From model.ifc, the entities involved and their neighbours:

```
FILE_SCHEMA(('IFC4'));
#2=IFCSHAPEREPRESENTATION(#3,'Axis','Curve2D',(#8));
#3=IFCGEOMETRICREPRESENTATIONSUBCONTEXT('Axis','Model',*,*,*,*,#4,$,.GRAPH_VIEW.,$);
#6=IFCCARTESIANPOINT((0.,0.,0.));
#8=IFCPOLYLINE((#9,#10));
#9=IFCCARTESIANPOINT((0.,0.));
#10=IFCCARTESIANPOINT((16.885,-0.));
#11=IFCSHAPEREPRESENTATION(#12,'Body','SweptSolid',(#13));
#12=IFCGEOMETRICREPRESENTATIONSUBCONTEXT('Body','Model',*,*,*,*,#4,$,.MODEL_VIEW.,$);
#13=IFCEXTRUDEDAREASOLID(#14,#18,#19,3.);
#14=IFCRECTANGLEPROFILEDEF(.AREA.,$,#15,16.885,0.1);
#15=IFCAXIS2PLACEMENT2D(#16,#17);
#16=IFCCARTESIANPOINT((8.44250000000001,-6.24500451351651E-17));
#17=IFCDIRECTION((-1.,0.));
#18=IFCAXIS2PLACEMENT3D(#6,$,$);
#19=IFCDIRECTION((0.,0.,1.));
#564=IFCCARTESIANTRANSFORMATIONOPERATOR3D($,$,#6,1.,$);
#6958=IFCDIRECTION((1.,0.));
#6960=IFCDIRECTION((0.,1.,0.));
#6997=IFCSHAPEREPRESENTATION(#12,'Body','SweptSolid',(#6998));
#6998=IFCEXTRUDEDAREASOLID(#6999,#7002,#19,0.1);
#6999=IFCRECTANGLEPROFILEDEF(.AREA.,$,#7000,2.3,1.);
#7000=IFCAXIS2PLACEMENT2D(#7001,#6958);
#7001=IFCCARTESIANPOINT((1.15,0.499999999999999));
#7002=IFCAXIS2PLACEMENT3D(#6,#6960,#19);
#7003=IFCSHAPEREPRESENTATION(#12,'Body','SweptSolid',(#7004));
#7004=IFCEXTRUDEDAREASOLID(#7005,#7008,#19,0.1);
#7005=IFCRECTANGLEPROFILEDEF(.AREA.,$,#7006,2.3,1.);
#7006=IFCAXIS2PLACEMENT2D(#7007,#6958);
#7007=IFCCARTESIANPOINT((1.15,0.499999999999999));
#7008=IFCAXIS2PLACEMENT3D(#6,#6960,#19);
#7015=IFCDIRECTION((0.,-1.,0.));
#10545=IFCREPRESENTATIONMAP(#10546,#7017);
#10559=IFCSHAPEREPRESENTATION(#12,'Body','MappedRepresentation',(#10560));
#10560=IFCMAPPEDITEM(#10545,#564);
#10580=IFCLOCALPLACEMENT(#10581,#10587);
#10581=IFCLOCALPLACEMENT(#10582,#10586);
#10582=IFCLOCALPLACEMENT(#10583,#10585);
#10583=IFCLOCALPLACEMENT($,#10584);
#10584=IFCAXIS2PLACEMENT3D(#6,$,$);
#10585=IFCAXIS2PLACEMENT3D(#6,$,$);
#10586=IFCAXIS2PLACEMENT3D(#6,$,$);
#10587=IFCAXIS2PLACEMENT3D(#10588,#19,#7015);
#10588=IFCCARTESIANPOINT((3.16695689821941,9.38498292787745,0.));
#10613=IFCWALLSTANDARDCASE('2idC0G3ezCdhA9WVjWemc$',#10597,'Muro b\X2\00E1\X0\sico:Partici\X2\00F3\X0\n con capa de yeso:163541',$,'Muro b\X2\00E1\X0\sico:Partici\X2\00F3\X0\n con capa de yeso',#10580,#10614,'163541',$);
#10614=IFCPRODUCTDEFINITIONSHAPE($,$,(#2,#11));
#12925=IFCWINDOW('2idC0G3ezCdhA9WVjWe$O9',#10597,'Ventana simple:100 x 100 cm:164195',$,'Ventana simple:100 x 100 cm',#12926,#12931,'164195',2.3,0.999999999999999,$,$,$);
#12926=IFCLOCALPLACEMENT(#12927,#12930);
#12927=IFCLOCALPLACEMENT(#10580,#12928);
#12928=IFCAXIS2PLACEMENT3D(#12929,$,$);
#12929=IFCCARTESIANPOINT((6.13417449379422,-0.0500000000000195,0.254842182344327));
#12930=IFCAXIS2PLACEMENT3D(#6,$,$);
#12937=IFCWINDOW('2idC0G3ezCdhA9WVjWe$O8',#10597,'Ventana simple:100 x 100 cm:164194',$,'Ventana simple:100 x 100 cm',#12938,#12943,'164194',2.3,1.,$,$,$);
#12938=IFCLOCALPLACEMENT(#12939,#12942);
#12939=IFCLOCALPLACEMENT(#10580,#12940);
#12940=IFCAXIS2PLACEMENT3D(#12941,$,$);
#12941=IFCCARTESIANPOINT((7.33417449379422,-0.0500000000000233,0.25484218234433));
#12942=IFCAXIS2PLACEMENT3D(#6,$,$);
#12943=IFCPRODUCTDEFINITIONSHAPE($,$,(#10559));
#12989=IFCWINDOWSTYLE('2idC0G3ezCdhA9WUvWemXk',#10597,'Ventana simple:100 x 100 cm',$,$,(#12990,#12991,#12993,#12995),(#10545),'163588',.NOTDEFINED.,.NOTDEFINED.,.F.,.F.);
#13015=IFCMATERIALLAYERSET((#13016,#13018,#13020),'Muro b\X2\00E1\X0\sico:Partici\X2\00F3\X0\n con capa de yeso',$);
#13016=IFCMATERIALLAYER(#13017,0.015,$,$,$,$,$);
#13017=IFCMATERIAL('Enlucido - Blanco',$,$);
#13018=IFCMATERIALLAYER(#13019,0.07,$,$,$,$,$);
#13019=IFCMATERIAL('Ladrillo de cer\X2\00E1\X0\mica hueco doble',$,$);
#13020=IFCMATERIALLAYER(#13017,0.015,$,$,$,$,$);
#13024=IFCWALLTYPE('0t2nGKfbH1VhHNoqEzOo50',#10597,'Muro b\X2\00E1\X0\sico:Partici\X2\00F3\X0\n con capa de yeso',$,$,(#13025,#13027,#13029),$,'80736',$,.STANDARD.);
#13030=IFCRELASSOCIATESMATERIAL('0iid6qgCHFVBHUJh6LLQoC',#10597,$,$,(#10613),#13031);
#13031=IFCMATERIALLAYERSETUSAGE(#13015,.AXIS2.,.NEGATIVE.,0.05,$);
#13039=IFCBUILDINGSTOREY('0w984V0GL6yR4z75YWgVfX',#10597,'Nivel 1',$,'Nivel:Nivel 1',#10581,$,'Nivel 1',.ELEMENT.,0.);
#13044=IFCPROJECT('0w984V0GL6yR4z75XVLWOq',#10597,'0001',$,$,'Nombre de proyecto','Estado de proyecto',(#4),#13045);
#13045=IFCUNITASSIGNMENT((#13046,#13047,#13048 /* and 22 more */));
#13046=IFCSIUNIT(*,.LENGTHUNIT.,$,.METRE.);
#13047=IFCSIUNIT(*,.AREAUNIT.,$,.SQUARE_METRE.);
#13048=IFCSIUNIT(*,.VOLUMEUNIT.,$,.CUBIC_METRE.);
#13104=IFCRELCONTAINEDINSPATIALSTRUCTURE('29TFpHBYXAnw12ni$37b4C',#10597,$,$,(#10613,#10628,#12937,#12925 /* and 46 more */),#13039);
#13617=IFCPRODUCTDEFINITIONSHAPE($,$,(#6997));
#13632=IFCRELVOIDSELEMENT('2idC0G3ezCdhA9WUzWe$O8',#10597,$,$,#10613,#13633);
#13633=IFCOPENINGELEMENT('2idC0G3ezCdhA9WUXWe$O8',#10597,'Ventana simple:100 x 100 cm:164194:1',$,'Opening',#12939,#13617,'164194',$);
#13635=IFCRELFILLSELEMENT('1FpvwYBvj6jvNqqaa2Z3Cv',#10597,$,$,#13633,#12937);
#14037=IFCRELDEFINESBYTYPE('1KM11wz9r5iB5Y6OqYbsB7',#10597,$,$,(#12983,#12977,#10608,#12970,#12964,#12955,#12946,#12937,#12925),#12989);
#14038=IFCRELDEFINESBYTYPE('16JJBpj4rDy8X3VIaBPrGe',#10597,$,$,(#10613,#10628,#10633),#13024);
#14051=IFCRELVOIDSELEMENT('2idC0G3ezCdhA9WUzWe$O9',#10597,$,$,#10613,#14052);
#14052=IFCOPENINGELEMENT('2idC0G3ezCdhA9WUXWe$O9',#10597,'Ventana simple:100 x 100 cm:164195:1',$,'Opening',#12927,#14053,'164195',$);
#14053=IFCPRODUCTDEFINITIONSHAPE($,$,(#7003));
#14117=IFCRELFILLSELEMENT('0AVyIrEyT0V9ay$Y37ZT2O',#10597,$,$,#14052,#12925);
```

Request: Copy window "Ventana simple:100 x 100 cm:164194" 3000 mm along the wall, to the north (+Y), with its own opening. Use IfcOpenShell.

```python
import ifcopenshell
import ifcopenshell.api.feature
import ifcopenshell.api.geometry
import ifcopenshell.api.root
import ifcopenshell.geom
import ifcopenshell.util.element
import ifcopenshell.util.placement
import ifcopenshell.util.shape

model = ifcopenshell.open("model.ifc")
settings = ifcopenshell.geom.settings()


def volume(element):
    """Net volume in cubic metres, openings subtracted."""
    shape = ifcopenshell.geom.create_shape(settings, element)
    return ifcopenshell.util.shape.get_volume(shape.geometry)


def reuse_history(source, copy):
    """copy_class also copies each property set's owner history, people and application; keep the originals."""
    for rel in copy.IsDefinedBy:
        if rel.is_a("IfcRelDefinesByProperties") and (history := rel.RelatingPropertyDefinition.OwnerHistory):
            rel.RelatingPropertyDefinition.OwnerHistory = source.OwnerHistory
            ifcopenshell.util.element.remove_deep2(model, history)


window = model.by_guid("2idC0G3ezCdhA9WVjWe$O8")
opening = window.FillsVoids[0].RelatingOpeningElement
wall = opening.VoidsElements[0].RelatingBuildingElement
before = volume(wall)
shift = ifcopenshell.util.placement.get_local_placement(wall.ObjectPlacement)[:3, 0] * -3.0

# copy_class copies the void relationship, type, container and properties, but no geometry.
new_opening = ifcopenshell.api.root.copy_class(model, product=opening)
new_opening.Representation = ifcopenshell.util.element.copy_deep(
    model, opening.Representation, exclude=["IfcGeometricRepresentationContext", "IfcRepresentationMap"]
)
new_opening.Name = "Ventana simple:100 x 100 cm"
new_opening.Tag = None
new_window = ifcopenshell.api.root.copy_class(model, product=window)
new_window.Representation = ifcopenshell.util.element.copy_deep(
    model, window.Representation, exclude=["IfcGeometricRepresentationContext", "IfcRepresentationMap"]
)
new_window.Name = "Ventana simple:100 x 100 cm"
new_window.Tag = None
reuse_history(window, new_window)
ifcopenshell.api.feature.add_filling(model, opening=new_opening, element=new_window)

for old, new in ((opening, new_opening), (window, new_window)):
    matrix = ifcopenshell.util.placement.get_local_placement(old.ObjectPlacement)
    matrix[:3, 3] += shift
    ifcopenshell.api.geometry.edit_object_placement(model, product=new, matrix=matrix, is_si=False)

after = volume(wall)

print(f"wall volume {before:.3f} -> {after:.3f} m3")

model.write("model_updated.ifc")
```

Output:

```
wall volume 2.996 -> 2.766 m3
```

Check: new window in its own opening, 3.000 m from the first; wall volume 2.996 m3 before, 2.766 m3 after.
